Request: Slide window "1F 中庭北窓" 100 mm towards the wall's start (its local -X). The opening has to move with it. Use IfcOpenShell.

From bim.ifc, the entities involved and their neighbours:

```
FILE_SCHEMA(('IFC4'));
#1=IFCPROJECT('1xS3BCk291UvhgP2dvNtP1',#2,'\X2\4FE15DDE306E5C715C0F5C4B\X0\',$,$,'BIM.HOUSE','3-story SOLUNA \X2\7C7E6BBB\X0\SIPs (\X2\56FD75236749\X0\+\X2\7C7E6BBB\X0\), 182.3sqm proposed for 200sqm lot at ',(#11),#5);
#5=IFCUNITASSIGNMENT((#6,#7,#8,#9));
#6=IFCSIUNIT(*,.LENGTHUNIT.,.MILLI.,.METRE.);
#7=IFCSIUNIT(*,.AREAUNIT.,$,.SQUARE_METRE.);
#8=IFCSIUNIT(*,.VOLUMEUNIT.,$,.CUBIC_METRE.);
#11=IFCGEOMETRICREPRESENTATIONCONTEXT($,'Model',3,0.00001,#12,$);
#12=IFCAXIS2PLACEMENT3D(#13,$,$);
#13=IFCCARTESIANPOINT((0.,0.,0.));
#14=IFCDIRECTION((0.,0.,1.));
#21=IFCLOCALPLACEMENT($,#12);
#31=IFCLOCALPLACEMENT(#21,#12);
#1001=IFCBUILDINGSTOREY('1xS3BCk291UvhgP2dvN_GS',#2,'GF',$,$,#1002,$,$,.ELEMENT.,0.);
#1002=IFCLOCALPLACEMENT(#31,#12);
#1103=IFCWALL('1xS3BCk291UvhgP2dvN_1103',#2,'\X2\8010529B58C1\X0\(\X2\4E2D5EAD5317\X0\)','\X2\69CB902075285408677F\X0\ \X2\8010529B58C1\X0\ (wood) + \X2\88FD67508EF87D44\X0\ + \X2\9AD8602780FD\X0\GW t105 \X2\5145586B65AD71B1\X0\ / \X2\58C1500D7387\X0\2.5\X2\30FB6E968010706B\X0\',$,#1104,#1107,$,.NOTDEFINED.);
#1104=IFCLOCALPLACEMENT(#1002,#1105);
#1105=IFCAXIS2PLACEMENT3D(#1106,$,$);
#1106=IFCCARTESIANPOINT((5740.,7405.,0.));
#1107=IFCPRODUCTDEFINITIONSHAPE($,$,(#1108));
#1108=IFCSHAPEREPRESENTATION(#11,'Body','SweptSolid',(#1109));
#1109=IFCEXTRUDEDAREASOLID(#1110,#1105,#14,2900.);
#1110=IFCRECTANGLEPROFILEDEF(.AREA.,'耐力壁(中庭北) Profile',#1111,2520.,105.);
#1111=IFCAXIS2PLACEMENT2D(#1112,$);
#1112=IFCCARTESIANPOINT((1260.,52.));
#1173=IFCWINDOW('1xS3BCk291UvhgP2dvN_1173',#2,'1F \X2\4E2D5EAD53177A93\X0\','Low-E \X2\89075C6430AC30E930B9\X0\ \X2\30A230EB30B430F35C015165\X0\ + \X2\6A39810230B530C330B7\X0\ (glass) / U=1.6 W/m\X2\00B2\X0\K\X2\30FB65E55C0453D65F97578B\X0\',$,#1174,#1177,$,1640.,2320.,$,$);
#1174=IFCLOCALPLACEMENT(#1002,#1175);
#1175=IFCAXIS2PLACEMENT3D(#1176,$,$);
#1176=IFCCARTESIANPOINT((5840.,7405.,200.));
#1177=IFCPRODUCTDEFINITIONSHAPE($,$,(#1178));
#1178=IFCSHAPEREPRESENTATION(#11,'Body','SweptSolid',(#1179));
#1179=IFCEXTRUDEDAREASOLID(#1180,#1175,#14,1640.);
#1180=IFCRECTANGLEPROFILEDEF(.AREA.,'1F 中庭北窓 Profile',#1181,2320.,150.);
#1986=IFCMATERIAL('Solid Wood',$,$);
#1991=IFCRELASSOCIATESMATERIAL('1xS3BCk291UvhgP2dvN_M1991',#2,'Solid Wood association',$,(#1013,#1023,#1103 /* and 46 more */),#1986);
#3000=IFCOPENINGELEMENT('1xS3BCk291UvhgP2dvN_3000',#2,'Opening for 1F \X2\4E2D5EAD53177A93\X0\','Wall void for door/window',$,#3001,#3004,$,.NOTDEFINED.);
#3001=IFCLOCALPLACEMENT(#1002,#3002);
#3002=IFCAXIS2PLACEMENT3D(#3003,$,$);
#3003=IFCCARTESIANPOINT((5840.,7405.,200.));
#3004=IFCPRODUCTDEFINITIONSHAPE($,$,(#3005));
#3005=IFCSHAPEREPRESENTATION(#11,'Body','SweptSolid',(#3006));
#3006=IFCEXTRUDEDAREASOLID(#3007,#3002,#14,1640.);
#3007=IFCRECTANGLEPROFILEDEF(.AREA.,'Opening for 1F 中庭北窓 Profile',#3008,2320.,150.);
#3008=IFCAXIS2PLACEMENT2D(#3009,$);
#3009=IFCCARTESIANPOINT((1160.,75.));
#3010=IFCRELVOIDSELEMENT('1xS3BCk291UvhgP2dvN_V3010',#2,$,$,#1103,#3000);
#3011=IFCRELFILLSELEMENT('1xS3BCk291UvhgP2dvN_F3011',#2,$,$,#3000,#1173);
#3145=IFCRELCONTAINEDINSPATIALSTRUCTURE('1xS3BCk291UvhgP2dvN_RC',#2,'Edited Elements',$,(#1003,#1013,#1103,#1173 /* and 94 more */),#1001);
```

```python
import ifcopenshell
import ifcopenshell.api.geometry
import ifcopenshell.util.placement

model = ifcopenshell.open("bim.ifc")

window = model.by_guid("1xS3BCk291UvhgP2dvN_1173")
opening = window.FillsVoids[0].RelatingOpeningElement
wall = opening.VoidsElements[0].RelatingBuildingElement

wall_matrix = ifcopenshell.util.placement.get_local_placement(wall.ObjectPlacement)
shift = wall_matrix[:3, 0] * -100.0
before = ifcopenshell.util.placement.get_local_placement(window.ObjectPlacement)[:3, 3].copy()

# The window is not placed relative to its opening, so move both.
for product in (opening, window):
    matrix = ifcopenshell.util.placement.get_local_placement(product.ObjectPlacement)
    matrix[:3, 3] += shift
    ifcopenshell.api.geometry.edit_object_placement(model, product=product, matrix=matrix, is_si=False)

after = ifcopenshell.util.placement.get_local_placement(window.ObjectPlacement)[:3, 3]
print("window moved by", (after - before).round(3) + 0.0)

model.write("bim-out.ifc")
```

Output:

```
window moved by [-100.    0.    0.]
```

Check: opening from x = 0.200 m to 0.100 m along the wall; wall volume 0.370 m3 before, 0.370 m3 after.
